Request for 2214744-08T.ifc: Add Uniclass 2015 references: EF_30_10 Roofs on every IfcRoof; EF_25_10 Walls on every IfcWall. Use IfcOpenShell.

First a look at what the model holds.

```python
import ifcopenshell

model = ifcopenshell.open("2214744-08T.ifc")
print(model.schema)
print("classifications:", [c.Name for c in model.by_type("IfcClassification")])
for ifc_class in ("IfcDoor", "IfcRoof", "IfcStair", "IfcWall", "IfcWindow"):
    print(ifc_class, len(model.by_type(ifc_class)))
```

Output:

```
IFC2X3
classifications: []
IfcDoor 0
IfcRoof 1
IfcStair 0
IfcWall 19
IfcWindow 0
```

```python
import ifcopenshell
import ifcopenshell.api.classification

model = ifcopenshell.open("2214744-08T.ifc")

# IFC2X3 requires Source and Edition and has no link from the project to the system.
system = model.create_entity("IfcClassification", Source="NBS", Edition="2015", Name="Uniclass 2015")

codes = {
    "IfcRoof": ("EF_30_10", "Roofs"),
    "IfcWall": ("EF_25_10", "Walls"),
}
for ifc_class, (code, name) in codes.items():
    products = model.by_type(ifc_class)
    ifcopenshell.api.classification.add_reference(
        model, products=products, classification=system, identification=code, name=name
    )
    print(code, len(products))

model.write("2214744-08T_v2.ifc")
```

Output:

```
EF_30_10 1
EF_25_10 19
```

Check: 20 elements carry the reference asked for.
